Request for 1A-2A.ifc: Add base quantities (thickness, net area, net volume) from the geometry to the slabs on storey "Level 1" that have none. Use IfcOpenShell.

First a look at what the model holds.

```python
import ifcopenshell
import ifcopenshell.util.element
import ifcopenshell.util.unit

model = ifcopenshell.open("1A-2A.ifc")
print(model.schema)
for unit_type in ("LENGTHUNIT", "AREAUNIT", "VOLUMEUNIT"):
    print(unit_type, ifcopenshell.util.unit.calculate_unit_scale(model, unit_type))
storey = next(s for s in model.by_type("IfcBuildingStorey") if s.Name == "Level 1")
slabs = [e for e in ifcopenshell.util.element.get_decomposition(storey) if e.is_a("IfcSlab")]
for e in sorted(slabs, key=lambda e: e.id()):
    print(e.id(), e.is_a(), e.Name, list(ifcopenshell.util.element.get_psets(e, qtos_only=True)), sep=" | ")
```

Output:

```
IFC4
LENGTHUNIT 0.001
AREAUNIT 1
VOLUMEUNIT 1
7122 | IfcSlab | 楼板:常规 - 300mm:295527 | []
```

```python
import ifcopenshell
import ifcopenshell.api.pset
import ifcopenshell.geom
import ifcopenshell.util.element
import ifcopenshell.util.shape
import ifcopenshell.util.unit

model = ifcopenshell.open("1A-2A.ifc")
unit_scale = ifcopenshell.util.unit.calculate_unit_scale(model)
area_scale = ifcopenshell.util.unit.calculate_unit_scale(model, "AREAUNIT")
volume_scale = ifcopenshell.util.unit.calculate_unit_scale(model, "VOLUMEUNIT")
settings = ifcopenshell.geom.settings()

storey = next(s for s in model.by_type("IfcBuildingStorey") if s.Name == "Level 1")
slabs = [e for e in ifcopenshell.util.element.get_decomposition(storey) if e.is_a("IfcSlab")]

for e in sorted(slabs, key=lambda e: e.id()):
    if ifcopenshell.util.element.get_psets(e, qtos_only=True, should_inherit=False):
        continue
    # Geometry comes back in metres, in the element's own axes.
    shape = ifcopenshell.geom.create_shape(settings, e)
    values = {
        "Width": ifcopenshell.util.shape.get_z(shape.geometry) / unit_scale,
        "NetArea": ifcopenshell.util.shape.get_footprint_area(shape.geometry) / area_scale,
        "NetVolume": ifcopenshell.util.shape.get_volume(shape.geometry) / volume_scale,
    }
    qto = ifcopenshell.api.pset.add_qto(model, product=e, name="Qto_SlabBaseQuantities")
    ifcopenshell.api.pset.edit_qto(model, qto=qto, properties=values)
    print(e.id(), {k: round(v, 3) for k, v in values.items()})

model.write("1A-2A_updated.ifc")
```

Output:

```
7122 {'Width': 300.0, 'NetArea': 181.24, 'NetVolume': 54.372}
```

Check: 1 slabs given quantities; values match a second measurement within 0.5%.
